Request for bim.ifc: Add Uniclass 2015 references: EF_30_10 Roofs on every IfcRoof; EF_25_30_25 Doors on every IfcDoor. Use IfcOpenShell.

First a look at what the model holds.

```python
import ifcopenshell

model = ifcopenshell.open("bim.ifc")
print(model.schema)
print("classifications:", [c.Name for c in model.by_type("IfcClassification")])
for ifc_class in ("IfcDoor", "IfcRoof", "IfcStair", "IfcWall", "IfcWindow"):
    print(ifc_class, len(model.by_type(ifc_class)))
```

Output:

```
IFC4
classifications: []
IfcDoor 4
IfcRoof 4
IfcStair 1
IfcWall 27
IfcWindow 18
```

```python
import ifcopenshell
import ifcopenshell.api.classification

model = ifcopenshell.open("bim.ifc")

system = ifcopenshell.api.classification.add_classification(model, classification="Uniclass 2015")

codes = {
    "IfcRoof": ("EF_30_10", "Roofs"),
    "IfcDoor": ("EF_25_30_25", "Doors"),
}
for ifc_class, (code, name) in codes.items():
    products = model.by_type(ifc_class)
    ifcopenshell.api.classification.add_reference(
        model, products=products, classification=system, identification=code, name=name
    )
    print(code, len(products))

model.write("bim_v2.ifc")
```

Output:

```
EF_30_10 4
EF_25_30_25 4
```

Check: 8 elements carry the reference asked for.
